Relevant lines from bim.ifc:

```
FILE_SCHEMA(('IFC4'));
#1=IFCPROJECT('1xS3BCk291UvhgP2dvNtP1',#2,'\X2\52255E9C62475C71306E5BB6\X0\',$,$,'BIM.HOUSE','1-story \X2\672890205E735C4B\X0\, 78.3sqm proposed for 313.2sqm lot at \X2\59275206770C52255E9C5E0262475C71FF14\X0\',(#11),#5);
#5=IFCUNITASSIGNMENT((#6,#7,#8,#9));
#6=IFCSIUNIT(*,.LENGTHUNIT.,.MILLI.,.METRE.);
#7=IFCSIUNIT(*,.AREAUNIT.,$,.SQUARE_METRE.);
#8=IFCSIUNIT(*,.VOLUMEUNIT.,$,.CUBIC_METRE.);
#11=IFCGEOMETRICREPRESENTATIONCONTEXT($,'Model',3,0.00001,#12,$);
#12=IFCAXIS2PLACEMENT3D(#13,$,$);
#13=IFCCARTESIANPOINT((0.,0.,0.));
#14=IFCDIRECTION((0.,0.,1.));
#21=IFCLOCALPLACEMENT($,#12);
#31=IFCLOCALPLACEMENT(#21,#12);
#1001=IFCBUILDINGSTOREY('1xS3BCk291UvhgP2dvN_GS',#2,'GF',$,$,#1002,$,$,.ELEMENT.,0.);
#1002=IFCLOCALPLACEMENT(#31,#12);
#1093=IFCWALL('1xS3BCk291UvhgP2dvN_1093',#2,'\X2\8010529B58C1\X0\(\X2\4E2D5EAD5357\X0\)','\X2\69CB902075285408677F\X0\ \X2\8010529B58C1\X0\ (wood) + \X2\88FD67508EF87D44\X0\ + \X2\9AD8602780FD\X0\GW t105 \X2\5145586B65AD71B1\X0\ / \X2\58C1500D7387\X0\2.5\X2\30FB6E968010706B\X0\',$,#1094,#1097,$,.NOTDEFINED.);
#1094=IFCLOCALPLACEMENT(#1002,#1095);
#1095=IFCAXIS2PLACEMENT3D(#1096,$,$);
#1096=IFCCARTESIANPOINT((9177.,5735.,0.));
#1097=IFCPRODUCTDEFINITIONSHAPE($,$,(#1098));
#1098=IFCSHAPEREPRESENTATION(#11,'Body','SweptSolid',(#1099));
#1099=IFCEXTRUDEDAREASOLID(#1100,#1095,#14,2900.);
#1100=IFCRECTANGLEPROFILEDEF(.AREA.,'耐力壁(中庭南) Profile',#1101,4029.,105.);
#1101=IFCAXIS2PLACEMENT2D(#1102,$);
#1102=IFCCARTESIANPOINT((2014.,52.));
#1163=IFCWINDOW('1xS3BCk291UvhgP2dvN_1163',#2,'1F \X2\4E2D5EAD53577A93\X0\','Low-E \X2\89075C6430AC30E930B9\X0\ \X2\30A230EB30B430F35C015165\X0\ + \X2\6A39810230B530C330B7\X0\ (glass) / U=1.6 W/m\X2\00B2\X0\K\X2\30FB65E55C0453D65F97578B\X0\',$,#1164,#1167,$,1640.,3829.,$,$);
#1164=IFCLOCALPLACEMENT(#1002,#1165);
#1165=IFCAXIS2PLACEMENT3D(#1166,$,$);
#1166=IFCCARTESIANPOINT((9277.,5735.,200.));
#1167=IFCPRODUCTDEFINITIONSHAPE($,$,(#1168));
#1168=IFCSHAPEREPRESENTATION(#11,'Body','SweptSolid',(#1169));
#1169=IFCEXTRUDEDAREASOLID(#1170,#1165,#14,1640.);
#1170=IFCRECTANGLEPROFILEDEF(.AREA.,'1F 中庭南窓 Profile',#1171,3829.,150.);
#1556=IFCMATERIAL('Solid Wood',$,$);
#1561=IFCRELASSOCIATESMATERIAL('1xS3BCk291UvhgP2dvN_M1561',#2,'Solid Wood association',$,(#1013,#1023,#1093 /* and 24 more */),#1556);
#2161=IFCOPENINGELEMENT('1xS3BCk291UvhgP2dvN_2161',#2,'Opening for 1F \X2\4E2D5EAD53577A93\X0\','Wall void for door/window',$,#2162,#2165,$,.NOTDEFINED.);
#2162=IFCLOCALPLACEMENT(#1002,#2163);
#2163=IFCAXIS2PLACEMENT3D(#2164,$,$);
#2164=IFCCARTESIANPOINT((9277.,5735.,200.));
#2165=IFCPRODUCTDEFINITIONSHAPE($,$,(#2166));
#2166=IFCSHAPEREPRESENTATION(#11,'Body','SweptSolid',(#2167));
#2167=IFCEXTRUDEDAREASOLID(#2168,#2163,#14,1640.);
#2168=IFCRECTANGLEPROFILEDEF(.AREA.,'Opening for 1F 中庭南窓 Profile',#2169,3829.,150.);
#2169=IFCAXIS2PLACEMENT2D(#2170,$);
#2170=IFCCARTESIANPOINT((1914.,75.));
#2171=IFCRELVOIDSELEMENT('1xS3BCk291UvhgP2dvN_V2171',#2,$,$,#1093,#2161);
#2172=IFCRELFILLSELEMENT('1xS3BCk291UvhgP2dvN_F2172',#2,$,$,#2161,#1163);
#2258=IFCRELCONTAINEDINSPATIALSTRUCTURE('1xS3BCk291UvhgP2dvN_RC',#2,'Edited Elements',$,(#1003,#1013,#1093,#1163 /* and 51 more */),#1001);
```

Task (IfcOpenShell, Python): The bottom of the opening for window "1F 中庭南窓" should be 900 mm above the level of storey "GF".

```python
import numpy as np
import ifcopenshell
import ifcopenshell.api.geometry
import ifcopenshell.geom
import ifcopenshell.util.element
import ifcopenshell.util.placement
import ifcopenshell.util.shape
import ifcopenshell.util.unit

model = ifcopenshell.open("bim.ifc")
unit_scale = ifcopenshell.util.unit.calculate_unit_scale(model)

window = model.by_guid("1xS3BCk291UvhgP2dvN_1163")
opening = window.FillsVoids[0].RelatingOpeningElement
storey = ifcopenshell.util.element.get_container(window, ifc_class="IfcBuildingStorey")
level = ifcopenshell.util.placement.get_local_placement(storey.ObjectPlacement)[2, 3]

# The opening's origin need not be at the sill, so measure its lowest point.
shape = ifcopenshell.geom.create_shape(ifcopenshell.geom.settings(), opening)
bottom = ifcopenshell.util.shape.get_shape_bottom_elevation(shape, shape.geometry) / unit_scale
dz = level + 0.9 / unit_scale - bottom

shift = np.array([0.0, 0.0, dz])
# The window is not placed relative to its opening, so move both.
for product in (opening, window):
    matrix = ifcopenshell.util.placement.get_local_placement(product.ObjectPlacement)
    matrix[:3, 3] += shift
    ifcopenshell.api.geometry.edit_object_placement(model, product=product, matrix=matrix, is_si=False)

print(f"moved by {dz * unit_scale:+.3f} m")

model.write("bim_v2.ifc")
```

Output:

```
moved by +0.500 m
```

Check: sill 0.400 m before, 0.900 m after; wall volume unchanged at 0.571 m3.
